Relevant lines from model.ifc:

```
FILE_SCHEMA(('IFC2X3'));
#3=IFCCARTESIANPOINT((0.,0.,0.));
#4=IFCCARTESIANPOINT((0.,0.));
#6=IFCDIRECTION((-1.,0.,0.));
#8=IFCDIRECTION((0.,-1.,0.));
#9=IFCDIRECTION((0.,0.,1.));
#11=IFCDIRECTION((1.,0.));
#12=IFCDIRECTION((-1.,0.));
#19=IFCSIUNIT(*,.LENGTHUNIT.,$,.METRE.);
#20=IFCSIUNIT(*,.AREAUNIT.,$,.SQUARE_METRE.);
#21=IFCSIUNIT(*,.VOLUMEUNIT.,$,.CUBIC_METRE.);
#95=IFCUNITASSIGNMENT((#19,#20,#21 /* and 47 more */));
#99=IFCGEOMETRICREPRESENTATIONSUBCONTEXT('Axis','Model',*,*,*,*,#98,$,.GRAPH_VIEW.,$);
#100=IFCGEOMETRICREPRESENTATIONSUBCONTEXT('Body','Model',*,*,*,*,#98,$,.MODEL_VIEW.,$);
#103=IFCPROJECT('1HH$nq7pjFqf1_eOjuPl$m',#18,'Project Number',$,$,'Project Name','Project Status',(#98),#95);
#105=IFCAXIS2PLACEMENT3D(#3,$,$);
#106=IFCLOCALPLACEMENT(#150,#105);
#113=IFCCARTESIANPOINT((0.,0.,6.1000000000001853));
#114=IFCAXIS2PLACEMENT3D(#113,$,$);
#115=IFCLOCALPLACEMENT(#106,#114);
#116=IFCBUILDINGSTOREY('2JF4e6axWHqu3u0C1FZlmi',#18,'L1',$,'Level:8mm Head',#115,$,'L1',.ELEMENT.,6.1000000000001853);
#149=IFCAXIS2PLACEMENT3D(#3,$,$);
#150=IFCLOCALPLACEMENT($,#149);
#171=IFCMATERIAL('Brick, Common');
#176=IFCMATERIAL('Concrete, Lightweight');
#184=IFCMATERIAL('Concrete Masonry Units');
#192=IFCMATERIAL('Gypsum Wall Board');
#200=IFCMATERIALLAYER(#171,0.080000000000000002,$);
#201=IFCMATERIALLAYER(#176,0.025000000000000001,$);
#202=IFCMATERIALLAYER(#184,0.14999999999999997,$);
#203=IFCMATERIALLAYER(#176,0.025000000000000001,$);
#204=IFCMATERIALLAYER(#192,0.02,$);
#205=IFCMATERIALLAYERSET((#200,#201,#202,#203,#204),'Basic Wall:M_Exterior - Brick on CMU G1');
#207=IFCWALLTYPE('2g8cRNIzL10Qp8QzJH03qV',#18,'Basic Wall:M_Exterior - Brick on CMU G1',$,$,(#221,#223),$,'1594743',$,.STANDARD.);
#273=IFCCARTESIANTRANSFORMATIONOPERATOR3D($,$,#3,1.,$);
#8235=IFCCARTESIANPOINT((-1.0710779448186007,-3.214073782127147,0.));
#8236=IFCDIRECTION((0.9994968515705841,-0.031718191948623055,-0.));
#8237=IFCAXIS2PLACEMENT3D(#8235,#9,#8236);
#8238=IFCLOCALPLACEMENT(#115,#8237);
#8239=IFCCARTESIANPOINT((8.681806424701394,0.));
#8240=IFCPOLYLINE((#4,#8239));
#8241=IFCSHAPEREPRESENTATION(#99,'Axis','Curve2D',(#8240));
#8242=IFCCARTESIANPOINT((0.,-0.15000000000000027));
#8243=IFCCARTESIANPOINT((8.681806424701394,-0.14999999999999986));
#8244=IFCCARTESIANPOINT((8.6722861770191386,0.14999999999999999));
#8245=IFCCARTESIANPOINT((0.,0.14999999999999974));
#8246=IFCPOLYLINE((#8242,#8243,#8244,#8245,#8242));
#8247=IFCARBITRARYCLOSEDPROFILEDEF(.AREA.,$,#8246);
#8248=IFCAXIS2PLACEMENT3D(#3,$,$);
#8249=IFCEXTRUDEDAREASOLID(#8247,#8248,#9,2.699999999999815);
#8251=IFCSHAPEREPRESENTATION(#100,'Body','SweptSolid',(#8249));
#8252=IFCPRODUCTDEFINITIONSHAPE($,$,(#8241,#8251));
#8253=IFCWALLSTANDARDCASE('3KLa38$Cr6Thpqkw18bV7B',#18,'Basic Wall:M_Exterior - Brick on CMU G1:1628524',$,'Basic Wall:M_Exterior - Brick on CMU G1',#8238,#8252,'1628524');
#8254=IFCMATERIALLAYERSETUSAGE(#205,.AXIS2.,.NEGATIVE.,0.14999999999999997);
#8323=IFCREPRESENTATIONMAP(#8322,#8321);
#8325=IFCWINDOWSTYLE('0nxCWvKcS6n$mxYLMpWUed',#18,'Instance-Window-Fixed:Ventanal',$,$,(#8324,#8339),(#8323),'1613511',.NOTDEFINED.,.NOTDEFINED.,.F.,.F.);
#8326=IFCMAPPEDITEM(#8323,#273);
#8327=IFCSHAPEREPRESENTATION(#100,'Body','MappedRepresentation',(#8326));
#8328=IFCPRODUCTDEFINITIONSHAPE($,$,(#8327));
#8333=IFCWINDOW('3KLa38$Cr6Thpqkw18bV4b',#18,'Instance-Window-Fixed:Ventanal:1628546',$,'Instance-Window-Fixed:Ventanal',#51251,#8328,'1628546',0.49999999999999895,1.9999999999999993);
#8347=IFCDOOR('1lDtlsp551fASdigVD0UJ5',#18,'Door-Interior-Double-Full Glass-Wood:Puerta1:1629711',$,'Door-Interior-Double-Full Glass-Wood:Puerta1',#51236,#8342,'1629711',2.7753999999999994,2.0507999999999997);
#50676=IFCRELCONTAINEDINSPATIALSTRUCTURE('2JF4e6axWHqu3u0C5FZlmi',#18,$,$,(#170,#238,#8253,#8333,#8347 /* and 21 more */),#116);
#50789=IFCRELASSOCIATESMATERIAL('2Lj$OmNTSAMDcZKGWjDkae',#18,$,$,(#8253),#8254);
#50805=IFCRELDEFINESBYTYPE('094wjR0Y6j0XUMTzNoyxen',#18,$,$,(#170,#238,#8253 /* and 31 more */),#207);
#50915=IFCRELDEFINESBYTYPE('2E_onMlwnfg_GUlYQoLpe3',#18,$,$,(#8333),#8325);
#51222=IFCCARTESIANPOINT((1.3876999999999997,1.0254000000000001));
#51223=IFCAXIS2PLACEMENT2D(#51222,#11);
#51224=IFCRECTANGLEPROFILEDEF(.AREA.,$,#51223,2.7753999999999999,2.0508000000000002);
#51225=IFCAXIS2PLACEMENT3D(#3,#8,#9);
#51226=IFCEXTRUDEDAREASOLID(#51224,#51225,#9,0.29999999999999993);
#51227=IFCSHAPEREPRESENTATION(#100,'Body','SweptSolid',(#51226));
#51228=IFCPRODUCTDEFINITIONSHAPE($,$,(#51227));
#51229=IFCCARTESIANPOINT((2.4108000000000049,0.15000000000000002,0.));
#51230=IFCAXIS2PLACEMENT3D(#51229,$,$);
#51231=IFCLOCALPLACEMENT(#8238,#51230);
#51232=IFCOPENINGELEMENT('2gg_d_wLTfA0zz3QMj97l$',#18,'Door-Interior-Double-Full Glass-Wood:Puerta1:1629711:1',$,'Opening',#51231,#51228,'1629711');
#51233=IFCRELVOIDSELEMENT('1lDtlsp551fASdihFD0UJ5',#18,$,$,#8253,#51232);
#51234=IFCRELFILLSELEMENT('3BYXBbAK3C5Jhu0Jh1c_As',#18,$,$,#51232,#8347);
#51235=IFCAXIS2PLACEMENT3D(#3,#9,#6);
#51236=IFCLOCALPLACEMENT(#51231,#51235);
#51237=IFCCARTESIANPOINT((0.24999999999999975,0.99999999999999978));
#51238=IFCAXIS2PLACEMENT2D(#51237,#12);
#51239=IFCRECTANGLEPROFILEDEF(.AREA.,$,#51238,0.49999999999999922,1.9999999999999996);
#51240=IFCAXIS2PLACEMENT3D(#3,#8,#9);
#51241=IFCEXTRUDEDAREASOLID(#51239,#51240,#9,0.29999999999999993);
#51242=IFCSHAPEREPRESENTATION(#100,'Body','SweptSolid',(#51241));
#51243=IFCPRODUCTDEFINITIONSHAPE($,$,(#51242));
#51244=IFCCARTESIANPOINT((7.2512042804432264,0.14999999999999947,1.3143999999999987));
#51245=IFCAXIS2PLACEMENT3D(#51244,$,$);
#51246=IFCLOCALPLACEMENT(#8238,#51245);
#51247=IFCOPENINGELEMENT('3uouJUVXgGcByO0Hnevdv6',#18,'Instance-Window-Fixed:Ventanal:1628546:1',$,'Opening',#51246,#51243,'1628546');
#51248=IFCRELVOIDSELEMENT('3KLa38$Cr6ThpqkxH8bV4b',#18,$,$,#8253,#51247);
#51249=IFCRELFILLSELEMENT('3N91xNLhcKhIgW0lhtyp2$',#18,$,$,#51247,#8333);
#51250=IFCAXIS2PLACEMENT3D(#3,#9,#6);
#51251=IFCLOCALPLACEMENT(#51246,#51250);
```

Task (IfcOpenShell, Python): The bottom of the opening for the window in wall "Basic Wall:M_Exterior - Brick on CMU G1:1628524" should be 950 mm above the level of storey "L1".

```python
import numpy as np
import ifcopenshell
import ifcopenshell.api.geometry
import ifcopenshell.geom
import ifcopenshell.util.element
import ifcopenshell.util.placement
import ifcopenshell.util.shape
import ifcopenshell.util.unit

model = ifcopenshell.open("model.ifc")
unit_scale = ifcopenshell.util.unit.calculate_unit_scale(model)

window = model.by_guid("3KLa38$Cr6Thpqkw18bV4b")
opening = window.FillsVoids[0].RelatingOpeningElement
storey = ifcopenshell.util.element.get_container(window, ifc_class="IfcBuildingStorey")
level = ifcopenshell.util.placement.get_local_placement(storey.ObjectPlacement)[2, 3]

# The opening's origin need not be at the sill, so measure its lowest point.
shape = ifcopenshell.geom.create_shape(ifcopenshell.geom.settings(), opening)
bottom = ifcopenshell.util.shape.get_shape_bottom_elevation(shape, shape.geometry) / unit_scale
dz = level + 0.95 / unit_scale - bottom

shift = np.array([0.0, 0.0, dz])
# The window is placed relative to its opening, so it follows when the opening moves.
matrix = ifcopenshell.util.placement.get_local_placement(opening.ObjectPlacement)
matrix[:3, 3] += shift
ifcopenshell.api.geometry.edit_object_placement(
    model, product=opening, matrix=matrix, is_si=False, should_transform_children=True
)

print(f"moved by {dz * unit_scale:+.3f} m")

model.write("model_rev.ifc")
```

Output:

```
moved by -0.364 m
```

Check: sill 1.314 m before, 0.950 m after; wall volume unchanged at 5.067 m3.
